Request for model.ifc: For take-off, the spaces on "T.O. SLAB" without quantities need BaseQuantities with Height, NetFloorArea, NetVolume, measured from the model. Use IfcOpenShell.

First a look at what the model holds.

```python
import ifcopenshell
import ifcopenshell.util.element
import ifcopenshell.util.unit

model = ifcopenshell.open("model.ifc")
print(model.schema)
for unit_type in ("LENGTHUNIT", "AREAUNIT", "VOLUMEUNIT"):
    print(unit_type, ifcopenshell.util.unit.calculate_unit_scale(model, unit_type))
storey = next(s for s in model.by_type("IfcBuildingStorey") if s.Name == "T.O. SLAB")
spaces = [e for e in ifcopenshell.util.element.get_decomposition(storey) if e.is_a("IfcSpace")]
for e in sorted(spaces, key=lambda e: e.id()):
    print(e.id(), e.is_a(), e.Name, list(ifcopenshell.util.element.get_psets(e, qtos_only=True)), sep=" | ")
```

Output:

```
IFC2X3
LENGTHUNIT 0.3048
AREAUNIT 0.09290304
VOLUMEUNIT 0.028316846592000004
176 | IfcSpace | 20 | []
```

```python
import ifcopenshell
import ifcopenshell.api.pset
import ifcopenshell.geom
import ifcopenshell.util.element
import ifcopenshell.util.shape
import ifcopenshell.util.unit

model = ifcopenshell.open("model.ifc")
unit_scale = ifcopenshell.util.unit.calculate_unit_scale(model)
area_scale = ifcopenshell.util.unit.calculate_unit_scale(model, "AREAUNIT")
volume_scale = ifcopenshell.util.unit.calculate_unit_scale(model, "VOLUMEUNIT")
settings = ifcopenshell.geom.settings()

storey = next(s for s in model.by_type("IfcBuildingStorey") if s.Name == "T.O. SLAB")
spaces = [e for e in ifcopenshell.util.element.get_decomposition(storey) if e.is_a("IfcSpace")]

for e in sorted(spaces, key=lambda e: e.id()):
    if ifcopenshell.util.element.get_psets(e, qtos_only=True, should_inherit=False):
        continue
    # Geometry comes back in metres, in the element's own axes.
    shape = ifcopenshell.geom.create_shape(settings, e)
    values = {
        "Height": ifcopenshell.util.shape.get_z(shape.geometry) / unit_scale,
        "NetFloorArea": ifcopenshell.util.shape.get_footprint_area(shape.geometry) / area_scale,
        "NetVolume": ifcopenshell.util.shape.get_volume(shape.geometry) / volume_scale,
    }
    qto = ifcopenshell.api.pset.add_qto(model, product=e, name="BaseQuantities")
    ifcopenshell.api.pset.edit_qto(model, qto=qto, properties=values)
    print(e.id(), {k: round(v, 3) for k, v in values.items()})

model.write("model_updated.ifc")
```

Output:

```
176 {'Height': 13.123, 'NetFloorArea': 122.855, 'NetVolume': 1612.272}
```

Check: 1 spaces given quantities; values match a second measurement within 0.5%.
